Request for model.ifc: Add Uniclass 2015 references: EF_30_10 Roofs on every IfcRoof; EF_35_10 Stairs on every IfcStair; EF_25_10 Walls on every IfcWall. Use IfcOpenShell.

First a look at what the model holds.

```python
import ifcopenshell

model = ifcopenshell.open("model.ifc")
print(model.schema)
print("classifications:", [c.Name for c in model.by_type("IfcClassification")])
for ifc_class in ("IfcDoor", "IfcRoof", "IfcStair", "IfcWall", "IfcWindow"):
    print(ifc_class, len(model.by_type(ifc_class)))
```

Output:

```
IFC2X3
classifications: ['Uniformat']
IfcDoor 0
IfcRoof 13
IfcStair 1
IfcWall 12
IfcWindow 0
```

```python
import ifcopenshell
import ifcopenshell.api.classification

model = ifcopenshell.open("model.ifc")

# IFC2X3 requires Source and Edition and has no link from the project to the system.
system = model.create_entity("IfcClassification", Source="NBS", Edition="2015", Name="Uniclass 2015")

codes = {
    "IfcRoof": ("EF_30_10", "Roofs"),
    "IfcStair": ("EF_35_10", "Stairs"),
    "IfcWall": ("EF_25_10", "Walls"),
}
for ifc_class, (code, name) in codes.items():
    products = model.by_type(ifc_class)
    ifcopenshell.api.classification.add_reference(
        model, products=products, classification=system, identification=code, name=name
    )
    print(code, len(products))

model.write("model_edited.ifc")
```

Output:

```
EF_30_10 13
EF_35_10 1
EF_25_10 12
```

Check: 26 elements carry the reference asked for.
